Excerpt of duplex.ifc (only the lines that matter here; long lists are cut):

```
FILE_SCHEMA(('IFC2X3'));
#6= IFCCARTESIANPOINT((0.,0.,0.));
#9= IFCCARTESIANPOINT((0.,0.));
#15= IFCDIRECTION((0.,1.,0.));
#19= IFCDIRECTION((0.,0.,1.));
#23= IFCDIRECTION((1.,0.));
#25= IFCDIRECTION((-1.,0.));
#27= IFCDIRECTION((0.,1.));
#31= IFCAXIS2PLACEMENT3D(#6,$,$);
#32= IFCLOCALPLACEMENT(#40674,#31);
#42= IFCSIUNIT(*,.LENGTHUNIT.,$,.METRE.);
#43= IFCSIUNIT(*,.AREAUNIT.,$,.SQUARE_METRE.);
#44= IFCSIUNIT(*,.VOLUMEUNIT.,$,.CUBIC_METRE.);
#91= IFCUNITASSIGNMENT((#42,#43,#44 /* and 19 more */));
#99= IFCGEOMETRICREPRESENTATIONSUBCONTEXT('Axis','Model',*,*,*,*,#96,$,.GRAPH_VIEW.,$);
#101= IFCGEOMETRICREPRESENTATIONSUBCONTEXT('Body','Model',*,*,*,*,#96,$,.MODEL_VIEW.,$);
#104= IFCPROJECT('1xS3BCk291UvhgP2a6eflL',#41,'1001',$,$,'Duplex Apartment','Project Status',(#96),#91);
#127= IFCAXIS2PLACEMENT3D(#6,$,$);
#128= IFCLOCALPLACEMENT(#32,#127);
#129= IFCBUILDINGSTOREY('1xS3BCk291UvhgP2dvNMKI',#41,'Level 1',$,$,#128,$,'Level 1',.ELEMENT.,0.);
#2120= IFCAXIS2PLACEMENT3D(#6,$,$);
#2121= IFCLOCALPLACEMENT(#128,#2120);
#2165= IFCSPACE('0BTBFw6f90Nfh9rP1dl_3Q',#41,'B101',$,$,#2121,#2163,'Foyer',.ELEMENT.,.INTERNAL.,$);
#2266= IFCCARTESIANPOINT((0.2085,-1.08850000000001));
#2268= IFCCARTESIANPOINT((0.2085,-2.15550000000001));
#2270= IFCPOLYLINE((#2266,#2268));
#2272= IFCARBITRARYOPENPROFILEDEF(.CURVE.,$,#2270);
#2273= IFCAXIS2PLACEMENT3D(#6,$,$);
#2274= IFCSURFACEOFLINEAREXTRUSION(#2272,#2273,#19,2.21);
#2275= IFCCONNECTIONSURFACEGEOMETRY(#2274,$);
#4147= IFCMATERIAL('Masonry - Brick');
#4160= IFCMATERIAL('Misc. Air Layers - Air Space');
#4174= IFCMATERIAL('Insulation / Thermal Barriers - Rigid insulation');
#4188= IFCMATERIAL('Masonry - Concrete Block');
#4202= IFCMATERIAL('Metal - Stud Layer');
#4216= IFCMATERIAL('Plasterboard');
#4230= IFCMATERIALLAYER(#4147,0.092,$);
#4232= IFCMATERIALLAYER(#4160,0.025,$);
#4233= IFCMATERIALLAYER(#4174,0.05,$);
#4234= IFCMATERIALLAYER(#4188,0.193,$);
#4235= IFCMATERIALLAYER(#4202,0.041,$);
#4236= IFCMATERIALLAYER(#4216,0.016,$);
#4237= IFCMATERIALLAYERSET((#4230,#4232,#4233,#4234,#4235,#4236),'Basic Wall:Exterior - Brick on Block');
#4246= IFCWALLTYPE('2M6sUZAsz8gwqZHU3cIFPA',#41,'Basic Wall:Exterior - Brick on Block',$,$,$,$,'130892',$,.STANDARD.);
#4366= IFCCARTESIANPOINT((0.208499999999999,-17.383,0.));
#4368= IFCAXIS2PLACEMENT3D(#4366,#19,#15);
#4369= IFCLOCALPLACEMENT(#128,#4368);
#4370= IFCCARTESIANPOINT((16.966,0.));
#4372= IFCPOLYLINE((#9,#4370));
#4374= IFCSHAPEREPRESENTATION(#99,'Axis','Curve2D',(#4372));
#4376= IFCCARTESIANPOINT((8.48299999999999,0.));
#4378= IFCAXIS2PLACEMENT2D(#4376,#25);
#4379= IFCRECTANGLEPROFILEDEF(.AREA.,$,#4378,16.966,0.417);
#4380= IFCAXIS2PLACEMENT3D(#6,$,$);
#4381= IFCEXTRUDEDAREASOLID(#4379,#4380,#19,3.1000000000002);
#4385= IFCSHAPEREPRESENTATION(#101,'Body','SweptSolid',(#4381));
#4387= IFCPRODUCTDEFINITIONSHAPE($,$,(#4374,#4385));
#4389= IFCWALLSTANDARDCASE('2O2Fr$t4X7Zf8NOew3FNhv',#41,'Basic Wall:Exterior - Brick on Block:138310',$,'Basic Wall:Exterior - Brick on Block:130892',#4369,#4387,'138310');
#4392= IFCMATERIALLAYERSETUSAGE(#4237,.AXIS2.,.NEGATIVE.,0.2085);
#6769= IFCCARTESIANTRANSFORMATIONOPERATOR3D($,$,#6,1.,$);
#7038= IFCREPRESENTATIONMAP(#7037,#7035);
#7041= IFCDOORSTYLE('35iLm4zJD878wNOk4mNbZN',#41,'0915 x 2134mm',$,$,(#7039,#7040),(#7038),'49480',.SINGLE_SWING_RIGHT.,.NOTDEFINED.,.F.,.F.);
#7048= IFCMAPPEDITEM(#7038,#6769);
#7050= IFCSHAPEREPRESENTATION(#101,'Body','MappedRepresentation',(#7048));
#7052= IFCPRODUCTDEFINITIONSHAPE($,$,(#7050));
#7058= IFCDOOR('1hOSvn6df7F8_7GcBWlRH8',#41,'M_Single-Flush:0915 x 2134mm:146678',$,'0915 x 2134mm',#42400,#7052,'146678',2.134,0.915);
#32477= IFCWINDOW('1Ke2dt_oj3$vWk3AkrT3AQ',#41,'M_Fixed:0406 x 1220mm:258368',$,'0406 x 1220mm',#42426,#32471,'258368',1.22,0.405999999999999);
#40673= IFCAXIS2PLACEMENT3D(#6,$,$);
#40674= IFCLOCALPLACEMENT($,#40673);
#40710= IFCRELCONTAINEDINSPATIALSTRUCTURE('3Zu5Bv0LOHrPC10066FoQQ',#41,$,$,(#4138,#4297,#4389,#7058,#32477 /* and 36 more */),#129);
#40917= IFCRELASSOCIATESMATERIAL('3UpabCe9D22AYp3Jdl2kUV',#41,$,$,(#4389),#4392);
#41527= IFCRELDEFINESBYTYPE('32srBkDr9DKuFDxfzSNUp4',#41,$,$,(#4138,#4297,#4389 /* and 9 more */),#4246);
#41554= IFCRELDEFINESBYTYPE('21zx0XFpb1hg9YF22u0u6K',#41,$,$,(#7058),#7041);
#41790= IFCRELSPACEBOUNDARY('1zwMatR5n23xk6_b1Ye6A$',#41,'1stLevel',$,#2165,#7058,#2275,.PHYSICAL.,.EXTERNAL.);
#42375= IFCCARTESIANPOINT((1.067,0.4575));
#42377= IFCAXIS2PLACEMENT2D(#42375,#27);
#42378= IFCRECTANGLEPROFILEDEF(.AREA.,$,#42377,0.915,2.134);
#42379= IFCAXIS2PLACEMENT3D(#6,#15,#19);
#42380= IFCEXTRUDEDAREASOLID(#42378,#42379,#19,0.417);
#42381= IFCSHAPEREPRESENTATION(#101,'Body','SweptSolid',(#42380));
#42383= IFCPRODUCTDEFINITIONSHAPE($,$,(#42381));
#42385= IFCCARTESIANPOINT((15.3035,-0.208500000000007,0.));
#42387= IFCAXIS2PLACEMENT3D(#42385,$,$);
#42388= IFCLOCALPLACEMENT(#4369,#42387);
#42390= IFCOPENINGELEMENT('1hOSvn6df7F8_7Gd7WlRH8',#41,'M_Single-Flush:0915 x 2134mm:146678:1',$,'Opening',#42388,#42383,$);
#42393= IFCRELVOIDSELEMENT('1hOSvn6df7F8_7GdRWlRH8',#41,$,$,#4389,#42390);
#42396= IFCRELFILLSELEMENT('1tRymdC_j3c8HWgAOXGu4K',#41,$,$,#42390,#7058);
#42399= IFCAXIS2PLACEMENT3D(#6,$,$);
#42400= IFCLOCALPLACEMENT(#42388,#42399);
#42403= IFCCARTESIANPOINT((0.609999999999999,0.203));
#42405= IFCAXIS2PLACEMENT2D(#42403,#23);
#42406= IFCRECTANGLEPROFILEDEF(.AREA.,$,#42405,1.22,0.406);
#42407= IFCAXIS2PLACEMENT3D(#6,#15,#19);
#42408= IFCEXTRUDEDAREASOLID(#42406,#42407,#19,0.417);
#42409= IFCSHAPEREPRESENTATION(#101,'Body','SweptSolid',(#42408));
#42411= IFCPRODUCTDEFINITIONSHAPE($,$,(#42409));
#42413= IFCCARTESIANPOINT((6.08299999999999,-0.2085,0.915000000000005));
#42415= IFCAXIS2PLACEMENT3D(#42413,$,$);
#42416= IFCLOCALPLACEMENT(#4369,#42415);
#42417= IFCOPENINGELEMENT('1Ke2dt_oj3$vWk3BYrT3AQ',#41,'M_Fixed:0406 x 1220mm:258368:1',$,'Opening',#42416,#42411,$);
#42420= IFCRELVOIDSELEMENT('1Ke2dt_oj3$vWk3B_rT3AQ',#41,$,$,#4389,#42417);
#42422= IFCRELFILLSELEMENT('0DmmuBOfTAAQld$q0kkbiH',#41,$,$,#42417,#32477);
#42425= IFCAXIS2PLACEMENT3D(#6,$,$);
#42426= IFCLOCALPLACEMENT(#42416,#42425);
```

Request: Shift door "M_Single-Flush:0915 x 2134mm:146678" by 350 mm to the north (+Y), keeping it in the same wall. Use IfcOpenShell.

```python
import numpy as np
import ifcopenshell
import ifcopenshell.api.geometry
import ifcopenshell.util.placement
import ifcopenshell.util.unit

model = ifcopenshell.open("duplex.ifc")
unit_scale = ifcopenshell.util.unit.calculate_unit_scale(model)

door = model.by_id(7058)
opening = door.FillsVoids[0].RelatingOpeningElement
wall = opening.VoidsElements[0].RelatingBuildingElement

wall_matrix = ifcopenshell.util.placement.get_local_placement(wall.ObjectPlacement)
shift = wall_matrix[:3, 0] * 0.35 / unit_scale
before = ifcopenshell.util.placement.get_local_placement(door.ObjectPlacement)[:3, 3].copy()

# The door is placed relative to its opening, so it follows when the opening moves.
matrix = ifcopenshell.util.placement.get_local_placement(opening.ObjectPlacement)
matrix[:3, 3] += shift
ifcopenshell.api.geometry.edit_object_placement(
    model, product=opening, matrix=matrix, is_si=False, should_transform_children=True
)

# Space boundary surfaces are stored in each space's coordinates; move them too.
for rel in door.ProvidesBoundaries:
    if not rel.ConnectionGeometry:
        continue
    surface = rel.ConnectionGeometry.SurfaceOnRelatingElement
    space_matrix = ifcopenshell.util.placement.get_local_placement(rel.RelatingSpace.ObjectPlacement)
    point = np.array(surface.Position.Location.Coordinates) + space_matrix[:3, :3].T @ shift
    surface.Position = model.createIfcAxis2Placement3D(
        model.createIfcCartesianPoint(point.tolist()), surface.Position.Axis, surface.Position.RefDirection
    )

after = ifcopenshell.util.placement.get_local_placement(door.ObjectPlacement)[:3, 3]
print("door moved by", (after - before).round(3) + 0.0)

model.write("duplex_edited.ifc")
```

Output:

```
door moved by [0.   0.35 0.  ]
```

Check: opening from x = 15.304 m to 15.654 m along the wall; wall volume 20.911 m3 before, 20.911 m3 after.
